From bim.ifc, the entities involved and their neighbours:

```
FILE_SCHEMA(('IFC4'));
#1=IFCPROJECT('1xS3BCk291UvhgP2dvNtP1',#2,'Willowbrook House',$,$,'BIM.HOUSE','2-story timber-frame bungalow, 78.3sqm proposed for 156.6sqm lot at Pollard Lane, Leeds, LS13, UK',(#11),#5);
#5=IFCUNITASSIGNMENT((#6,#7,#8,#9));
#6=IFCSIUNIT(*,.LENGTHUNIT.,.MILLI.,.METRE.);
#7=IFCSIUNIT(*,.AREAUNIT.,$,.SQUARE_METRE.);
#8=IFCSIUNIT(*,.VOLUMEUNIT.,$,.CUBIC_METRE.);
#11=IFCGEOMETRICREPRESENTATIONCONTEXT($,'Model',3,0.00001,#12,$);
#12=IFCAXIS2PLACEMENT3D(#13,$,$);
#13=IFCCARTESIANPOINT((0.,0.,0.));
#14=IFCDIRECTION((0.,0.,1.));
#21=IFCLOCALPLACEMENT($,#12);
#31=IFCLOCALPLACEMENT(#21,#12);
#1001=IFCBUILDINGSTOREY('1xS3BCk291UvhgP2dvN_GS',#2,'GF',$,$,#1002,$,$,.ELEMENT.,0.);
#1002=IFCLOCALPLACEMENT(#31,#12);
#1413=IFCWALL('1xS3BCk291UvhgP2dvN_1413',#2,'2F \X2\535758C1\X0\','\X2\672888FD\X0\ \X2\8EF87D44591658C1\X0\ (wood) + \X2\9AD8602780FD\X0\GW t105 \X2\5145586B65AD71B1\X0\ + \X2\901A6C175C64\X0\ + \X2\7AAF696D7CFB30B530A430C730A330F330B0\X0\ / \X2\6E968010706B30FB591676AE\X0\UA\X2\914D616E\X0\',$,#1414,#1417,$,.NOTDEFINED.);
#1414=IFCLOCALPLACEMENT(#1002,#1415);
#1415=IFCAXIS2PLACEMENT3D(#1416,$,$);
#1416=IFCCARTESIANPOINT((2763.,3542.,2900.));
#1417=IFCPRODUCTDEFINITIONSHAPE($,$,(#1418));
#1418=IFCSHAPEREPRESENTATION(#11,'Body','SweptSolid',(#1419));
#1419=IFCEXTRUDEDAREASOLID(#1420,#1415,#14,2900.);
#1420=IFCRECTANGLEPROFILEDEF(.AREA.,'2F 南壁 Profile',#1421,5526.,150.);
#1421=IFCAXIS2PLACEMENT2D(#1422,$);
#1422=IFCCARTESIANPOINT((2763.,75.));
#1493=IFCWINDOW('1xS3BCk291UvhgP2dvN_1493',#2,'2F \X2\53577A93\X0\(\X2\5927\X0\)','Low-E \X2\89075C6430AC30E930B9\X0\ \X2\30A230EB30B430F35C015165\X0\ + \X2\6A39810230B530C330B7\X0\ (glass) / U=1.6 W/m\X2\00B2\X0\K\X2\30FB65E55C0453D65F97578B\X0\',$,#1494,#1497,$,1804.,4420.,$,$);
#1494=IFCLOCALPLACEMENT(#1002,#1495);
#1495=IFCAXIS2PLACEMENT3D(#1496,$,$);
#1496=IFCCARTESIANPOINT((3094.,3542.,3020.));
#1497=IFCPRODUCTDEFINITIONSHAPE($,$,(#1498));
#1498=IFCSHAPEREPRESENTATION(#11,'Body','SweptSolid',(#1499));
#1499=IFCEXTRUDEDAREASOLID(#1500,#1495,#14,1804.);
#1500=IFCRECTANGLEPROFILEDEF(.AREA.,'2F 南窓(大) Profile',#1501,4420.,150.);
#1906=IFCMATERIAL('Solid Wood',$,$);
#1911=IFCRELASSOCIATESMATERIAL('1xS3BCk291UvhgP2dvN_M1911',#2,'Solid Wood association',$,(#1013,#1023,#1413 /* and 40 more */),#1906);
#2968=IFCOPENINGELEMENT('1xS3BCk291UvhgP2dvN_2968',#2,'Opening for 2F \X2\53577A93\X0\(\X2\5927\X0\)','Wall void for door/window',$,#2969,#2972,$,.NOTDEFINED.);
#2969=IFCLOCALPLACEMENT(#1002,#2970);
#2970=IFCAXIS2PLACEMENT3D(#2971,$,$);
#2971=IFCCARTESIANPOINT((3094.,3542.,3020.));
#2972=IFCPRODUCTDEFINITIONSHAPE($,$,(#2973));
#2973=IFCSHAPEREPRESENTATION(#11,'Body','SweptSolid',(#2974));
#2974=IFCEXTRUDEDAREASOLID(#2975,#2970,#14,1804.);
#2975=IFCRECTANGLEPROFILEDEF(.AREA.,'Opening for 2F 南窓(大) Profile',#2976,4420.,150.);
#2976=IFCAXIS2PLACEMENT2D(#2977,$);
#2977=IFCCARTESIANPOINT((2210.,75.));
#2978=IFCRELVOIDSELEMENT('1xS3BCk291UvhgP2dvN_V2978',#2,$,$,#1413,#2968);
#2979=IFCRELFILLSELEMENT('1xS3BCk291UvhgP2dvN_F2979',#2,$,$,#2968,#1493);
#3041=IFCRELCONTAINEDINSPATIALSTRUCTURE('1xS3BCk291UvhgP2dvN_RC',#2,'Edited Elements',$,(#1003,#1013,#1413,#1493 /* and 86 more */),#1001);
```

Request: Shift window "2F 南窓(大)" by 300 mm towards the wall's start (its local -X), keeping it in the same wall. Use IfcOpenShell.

```python
import ifcopenshell
import ifcopenshell.api.geometry
import ifcopenshell.util.placement
import ifcopenshell.util.unit

model = ifcopenshell.open("bim.ifc")
unit_scale = ifcopenshell.util.unit.calculate_unit_scale(model)

window = model.by_guid("1xS3BCk291UvhgP2dvN_1493")
opening = window.FillsVoids[0].RelatingOpeningElement
wall = opening.VoidsElements[0].RelatingBuildingElement

wall_matrix = ifcopenshell.util.placement.get_local_placement(wall.ObjectPlacement)
shift = wall_matrix[:3, 0] * -0.3 / unit_scale
before = ifcopenshell.util.placement.get_local_placement(window.ObjectPlacement)[:3, 3].copy()

# The window is not placed relative to its opening, so move both.
for product in (opening, window):
    matrix = ifcopenshell.util.placement.get_local_placement(product.ObjectPlacement)
    matrix[:3, 3] += shift
    ifcopenshell.api.geometry.edit_object_placement(model, product=product, matrix=matrix, is_si=False)

after = ifcopenshell.util.placement.get_local_placement(window.ObjectPlacement)[:3, 3]
print("window moved by", (after - before).round(3) + 0.0)

model.write("bim_rev.ifc")
```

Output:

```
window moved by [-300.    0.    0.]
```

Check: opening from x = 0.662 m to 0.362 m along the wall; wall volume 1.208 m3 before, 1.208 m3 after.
